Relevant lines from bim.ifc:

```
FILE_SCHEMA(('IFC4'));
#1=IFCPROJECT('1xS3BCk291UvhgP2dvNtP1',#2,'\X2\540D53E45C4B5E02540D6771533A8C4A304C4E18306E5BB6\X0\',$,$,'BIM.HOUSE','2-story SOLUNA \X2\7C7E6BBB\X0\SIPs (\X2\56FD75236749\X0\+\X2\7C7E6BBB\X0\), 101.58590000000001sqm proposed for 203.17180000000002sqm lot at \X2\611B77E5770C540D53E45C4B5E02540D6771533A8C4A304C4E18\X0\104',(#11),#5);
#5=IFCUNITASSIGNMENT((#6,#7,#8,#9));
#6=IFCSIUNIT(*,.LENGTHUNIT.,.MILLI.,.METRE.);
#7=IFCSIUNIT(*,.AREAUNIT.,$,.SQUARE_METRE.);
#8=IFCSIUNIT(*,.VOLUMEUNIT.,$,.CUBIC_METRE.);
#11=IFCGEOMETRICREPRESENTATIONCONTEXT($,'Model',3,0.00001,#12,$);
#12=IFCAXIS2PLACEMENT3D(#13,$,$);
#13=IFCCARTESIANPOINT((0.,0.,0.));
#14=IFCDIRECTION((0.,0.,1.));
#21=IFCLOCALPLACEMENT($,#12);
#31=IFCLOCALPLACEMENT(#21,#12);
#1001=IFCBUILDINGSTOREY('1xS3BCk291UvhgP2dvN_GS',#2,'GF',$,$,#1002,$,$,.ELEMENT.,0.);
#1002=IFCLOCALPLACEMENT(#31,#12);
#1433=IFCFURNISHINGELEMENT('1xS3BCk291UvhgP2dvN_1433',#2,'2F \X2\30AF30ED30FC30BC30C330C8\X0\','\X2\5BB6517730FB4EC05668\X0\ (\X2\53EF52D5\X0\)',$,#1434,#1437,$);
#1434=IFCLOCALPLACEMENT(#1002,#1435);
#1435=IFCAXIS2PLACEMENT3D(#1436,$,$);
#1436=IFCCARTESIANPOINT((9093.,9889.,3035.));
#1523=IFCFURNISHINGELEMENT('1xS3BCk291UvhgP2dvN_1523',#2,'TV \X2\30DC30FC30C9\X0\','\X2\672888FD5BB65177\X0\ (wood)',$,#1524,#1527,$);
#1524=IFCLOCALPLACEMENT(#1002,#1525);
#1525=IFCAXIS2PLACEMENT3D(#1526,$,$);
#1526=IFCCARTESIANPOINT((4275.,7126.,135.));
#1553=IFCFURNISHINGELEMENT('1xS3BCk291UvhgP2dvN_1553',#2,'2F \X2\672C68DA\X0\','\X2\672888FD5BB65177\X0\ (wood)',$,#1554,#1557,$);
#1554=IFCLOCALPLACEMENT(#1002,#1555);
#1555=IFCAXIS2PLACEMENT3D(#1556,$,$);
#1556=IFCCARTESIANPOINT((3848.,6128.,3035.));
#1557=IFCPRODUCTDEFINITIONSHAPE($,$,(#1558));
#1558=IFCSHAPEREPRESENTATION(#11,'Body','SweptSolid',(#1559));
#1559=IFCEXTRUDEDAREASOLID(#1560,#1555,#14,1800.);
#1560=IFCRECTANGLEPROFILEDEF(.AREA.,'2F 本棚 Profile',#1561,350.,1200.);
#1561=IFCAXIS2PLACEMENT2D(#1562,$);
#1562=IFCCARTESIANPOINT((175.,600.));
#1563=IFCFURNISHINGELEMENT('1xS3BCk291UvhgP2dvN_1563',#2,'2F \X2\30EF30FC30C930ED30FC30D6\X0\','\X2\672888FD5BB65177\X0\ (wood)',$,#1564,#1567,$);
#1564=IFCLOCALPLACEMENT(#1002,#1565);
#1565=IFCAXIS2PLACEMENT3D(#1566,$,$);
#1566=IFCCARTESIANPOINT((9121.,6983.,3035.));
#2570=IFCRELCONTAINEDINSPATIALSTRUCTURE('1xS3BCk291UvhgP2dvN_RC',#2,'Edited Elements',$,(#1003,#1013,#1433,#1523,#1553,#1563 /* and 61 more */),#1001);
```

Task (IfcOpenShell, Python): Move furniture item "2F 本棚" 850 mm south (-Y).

```python
import ifcopenshell
import ifcopenshell.api.geometry
import ifcopenshell.util.placement

model = ifcopenshell.open("bim.ifc")

item = model.by_guid("1xS3BCk291UvhgP2dvN_1553")
matrix = ifcopenshell.util.placement.get_local_placement(item.ObjectPlacement)
matrix[1, 3] -= 850.0
ifcopenshell.api.geometry.edit_object_placement(model, product=item, matrix=matrix, is_si=False)

print(ifcopenshell.util.placement.get_local_placement(item.ObjectPlacement).round(3) + 0.0)

model.write("bim_v2.ifc")
```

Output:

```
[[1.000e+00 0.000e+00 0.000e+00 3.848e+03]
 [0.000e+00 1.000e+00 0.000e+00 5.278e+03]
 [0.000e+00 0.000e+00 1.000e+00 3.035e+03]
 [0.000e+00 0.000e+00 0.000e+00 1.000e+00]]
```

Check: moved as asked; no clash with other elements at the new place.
